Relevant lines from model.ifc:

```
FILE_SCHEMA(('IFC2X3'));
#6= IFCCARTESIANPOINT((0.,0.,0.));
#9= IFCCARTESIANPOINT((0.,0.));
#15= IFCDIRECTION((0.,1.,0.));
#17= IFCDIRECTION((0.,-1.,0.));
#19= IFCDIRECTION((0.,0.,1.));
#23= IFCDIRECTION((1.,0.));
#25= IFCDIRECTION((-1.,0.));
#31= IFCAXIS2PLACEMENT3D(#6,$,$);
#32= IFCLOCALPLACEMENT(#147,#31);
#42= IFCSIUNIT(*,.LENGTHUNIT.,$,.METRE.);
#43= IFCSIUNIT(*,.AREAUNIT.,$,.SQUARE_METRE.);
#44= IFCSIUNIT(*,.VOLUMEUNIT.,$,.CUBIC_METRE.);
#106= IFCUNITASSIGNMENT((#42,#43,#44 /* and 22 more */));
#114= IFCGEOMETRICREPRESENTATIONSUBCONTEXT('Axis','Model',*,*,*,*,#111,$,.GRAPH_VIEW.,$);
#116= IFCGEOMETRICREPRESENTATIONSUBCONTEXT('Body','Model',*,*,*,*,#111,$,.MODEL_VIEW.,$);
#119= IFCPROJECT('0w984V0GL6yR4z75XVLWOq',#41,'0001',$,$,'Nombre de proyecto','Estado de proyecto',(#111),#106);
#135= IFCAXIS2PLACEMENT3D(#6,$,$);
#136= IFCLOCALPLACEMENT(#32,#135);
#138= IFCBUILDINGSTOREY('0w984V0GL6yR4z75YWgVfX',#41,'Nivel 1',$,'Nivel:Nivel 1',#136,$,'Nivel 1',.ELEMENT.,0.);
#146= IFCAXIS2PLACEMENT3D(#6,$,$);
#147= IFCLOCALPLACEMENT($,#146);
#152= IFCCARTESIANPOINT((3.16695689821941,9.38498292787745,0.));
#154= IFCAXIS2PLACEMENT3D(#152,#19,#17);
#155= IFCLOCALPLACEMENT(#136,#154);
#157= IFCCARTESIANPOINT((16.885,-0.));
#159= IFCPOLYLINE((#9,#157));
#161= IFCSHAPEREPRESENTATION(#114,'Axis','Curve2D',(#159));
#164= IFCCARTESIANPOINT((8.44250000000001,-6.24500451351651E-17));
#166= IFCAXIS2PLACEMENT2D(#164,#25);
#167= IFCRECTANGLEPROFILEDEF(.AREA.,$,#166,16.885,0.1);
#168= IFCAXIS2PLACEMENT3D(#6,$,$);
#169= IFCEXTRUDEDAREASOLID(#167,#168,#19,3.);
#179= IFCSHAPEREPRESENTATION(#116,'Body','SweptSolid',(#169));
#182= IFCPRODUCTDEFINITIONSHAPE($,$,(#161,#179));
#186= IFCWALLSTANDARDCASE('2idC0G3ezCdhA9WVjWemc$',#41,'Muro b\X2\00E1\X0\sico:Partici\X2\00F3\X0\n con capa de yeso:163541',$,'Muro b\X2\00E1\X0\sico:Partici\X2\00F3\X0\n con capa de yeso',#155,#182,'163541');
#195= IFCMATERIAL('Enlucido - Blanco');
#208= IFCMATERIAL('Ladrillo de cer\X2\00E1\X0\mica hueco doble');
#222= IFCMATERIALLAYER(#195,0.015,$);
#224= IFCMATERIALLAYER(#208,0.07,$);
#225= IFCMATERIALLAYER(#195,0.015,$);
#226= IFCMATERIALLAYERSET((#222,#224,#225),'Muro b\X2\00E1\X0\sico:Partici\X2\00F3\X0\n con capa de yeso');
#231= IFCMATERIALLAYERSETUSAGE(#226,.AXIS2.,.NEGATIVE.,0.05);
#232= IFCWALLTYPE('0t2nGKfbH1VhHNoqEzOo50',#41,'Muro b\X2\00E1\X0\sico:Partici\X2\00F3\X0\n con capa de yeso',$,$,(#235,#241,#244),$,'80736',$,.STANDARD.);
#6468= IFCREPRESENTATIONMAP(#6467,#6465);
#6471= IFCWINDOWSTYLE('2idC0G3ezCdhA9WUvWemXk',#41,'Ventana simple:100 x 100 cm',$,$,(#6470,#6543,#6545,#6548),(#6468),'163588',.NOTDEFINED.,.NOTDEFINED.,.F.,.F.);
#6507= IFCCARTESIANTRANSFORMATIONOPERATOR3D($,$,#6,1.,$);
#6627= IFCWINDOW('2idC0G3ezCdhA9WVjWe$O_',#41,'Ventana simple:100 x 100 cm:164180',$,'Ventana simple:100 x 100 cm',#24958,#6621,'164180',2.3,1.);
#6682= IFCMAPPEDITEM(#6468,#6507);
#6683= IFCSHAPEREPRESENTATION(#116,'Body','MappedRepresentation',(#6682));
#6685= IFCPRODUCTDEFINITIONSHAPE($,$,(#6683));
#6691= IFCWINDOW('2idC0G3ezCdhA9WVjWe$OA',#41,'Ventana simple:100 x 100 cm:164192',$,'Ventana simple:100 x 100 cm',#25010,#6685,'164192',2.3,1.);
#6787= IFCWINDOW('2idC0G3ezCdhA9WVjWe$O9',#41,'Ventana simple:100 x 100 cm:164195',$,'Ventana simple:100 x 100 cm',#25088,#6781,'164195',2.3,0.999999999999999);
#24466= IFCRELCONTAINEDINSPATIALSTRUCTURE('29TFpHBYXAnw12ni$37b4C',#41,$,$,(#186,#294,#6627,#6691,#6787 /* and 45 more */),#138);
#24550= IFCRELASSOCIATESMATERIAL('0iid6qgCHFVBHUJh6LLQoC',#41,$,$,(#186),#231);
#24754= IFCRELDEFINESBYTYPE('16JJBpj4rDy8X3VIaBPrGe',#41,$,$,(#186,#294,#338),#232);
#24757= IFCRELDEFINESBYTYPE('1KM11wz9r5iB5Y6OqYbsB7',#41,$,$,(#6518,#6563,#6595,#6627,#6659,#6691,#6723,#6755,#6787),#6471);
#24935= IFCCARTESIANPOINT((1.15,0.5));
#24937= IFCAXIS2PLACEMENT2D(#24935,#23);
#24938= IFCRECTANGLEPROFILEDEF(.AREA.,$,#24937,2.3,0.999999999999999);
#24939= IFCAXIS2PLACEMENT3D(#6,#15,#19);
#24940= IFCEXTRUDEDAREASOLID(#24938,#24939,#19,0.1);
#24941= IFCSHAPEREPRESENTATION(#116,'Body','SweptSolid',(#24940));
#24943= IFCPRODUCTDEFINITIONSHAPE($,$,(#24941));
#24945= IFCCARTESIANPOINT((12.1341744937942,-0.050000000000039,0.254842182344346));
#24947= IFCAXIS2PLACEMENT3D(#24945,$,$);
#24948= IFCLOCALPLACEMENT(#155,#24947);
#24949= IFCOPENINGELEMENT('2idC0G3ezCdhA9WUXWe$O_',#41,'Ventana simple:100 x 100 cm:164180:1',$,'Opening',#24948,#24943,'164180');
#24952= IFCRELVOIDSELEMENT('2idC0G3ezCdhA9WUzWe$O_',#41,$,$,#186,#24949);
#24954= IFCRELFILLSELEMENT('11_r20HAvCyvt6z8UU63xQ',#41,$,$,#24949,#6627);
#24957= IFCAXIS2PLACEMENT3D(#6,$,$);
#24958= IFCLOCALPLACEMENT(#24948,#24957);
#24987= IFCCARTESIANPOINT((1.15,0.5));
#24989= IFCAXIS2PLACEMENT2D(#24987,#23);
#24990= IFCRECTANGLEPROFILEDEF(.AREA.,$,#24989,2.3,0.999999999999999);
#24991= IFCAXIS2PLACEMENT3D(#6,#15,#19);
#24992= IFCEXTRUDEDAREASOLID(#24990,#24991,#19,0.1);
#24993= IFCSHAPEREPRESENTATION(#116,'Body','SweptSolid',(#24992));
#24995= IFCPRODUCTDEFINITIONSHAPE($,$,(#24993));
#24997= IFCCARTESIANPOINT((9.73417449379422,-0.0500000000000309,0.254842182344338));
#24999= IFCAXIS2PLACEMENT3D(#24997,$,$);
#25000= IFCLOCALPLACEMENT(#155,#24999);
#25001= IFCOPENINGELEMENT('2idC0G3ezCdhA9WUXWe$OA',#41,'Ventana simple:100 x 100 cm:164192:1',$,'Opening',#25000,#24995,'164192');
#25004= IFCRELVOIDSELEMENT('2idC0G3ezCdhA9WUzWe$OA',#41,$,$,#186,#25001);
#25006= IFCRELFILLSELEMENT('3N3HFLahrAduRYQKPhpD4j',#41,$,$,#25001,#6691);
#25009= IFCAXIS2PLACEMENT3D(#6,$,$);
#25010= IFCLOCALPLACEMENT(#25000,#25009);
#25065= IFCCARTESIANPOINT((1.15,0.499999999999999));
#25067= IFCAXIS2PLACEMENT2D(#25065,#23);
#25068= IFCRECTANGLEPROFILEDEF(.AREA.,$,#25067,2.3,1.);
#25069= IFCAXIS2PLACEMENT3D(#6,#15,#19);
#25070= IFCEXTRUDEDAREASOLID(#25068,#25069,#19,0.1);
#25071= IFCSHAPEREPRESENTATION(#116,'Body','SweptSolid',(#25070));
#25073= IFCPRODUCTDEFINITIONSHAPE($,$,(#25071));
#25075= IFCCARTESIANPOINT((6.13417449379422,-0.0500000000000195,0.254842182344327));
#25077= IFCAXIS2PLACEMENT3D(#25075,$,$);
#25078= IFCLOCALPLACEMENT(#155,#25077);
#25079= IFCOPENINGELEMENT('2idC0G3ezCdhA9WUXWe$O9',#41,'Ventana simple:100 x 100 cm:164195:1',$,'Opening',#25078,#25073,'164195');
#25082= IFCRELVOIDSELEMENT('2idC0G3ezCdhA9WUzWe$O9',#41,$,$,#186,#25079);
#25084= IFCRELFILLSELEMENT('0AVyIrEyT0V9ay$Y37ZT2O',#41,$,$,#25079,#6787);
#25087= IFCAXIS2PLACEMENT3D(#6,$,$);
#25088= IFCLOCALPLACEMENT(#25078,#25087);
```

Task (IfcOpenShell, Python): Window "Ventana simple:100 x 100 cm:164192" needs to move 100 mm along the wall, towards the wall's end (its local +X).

```python
import ifcopenshell
import ifcopenshell.api.geometry
import ifcopenshell.util.placement
import ifcopenshell.util.unit

model = ifcopenshell.open("model.ifc")
unit_scale = ifcopenshell.util.unit.calculate_unit_scale(model)

window = model.by_id(6691)
opening = window.FillsVoids[0].RelatingOpeningElement
wall = opening.VoidsElements[0].RelatingBuildingElement

wall_matrix = ifcopenshell.util.placement.get_local_placement(wall.ObjectPlacement)
shift = wall_matrix[:3, 0] * 0.1 / unit_scale
before = ifcopenshell.util.placement.get_local_placement(window.ObjectPlacement)[:3, 3].copy()

# The window is placed relative to its opening, so it follows when the opening moves.
matrix = ifcopenshell.util.placement.get_local_placement(opening.ObjectPlacement)
matrix[:3, 3] += shift
ifcopenshell.api.geometry.edit_object_placement(
    model, product=opening, matrix=matrix, is_si=False, should_transform_children=True
)

after = ifcopenshell.util.placement.get_local_placement(window.ObjectPlacement)[:3, 3]
print("window moved by", (after - before).round(3) + 0.0)

model.write("model-out.ifc")
```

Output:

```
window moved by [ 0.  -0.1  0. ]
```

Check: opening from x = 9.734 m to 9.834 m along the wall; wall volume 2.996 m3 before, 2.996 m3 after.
